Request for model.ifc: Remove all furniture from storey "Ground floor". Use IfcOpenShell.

First a look at what the model holds.

```python
import ifcopenshell
import ifcopenshell.util.element

model = ifcopenshell.open("model.ifc")
print(model.schema)
storey = next(s for s in model.by_type("IfcBuildingStorey") if s.Name == "Ground floor")
furniture = [e for e in ifcopenshell.util.element.get_decomposition(storey) if e.is_a("IfcFurnishingElement")]
seen = {}
for e in furniture:
    element_type = ifcopenshell.util.element.get_type(e)
    name = element_type.Name if element_type not in (None, e) else None
    seen[name] = seen.get(name, 0) + 1
for name, count in sorted(seen.items(), key=str):
    print(count, "x", name)
```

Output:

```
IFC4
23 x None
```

```python
import ifcopenshell
import ifcopenshell.api.root
import ifcopenshell.util.element

model = ifcopenshell.open("model.ifc")

storey = next(s for s in model.by_type("IfcBuildingStorey") if s.Name == "Ground floor")
furniture = [e for e in ifcopenshell.util.element.get_decomposition(storey) if e.is_a("IfcFurnishingElement")]

for e in furniture:
    ifcopenshell.api.root.remove_product(model, product=e)
print(len(furniture), "removed")

model.write("model_edited.ifc")
```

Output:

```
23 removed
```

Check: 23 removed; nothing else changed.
